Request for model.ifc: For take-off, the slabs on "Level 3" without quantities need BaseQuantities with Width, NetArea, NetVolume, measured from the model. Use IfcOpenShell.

First a look at what the model holds.

```python
import ifcopenshell
import ifcopenshell.util.element
import ifcopenshell.util.unit

model = ifcopenshell.open("model.ifc")
print(model.schema)
for unit_type in ("LENGTHUNIT", "AREAUNIT", "VOLUMEUNIT"):
    print(unit_type, ifcopenshell.util.unit.calculate_unit_scale(model, unit_type))
storey = next(s for s in model.by_type("IfcBuildingStorey") if s.Name == "Level 3")
slabs = [e for e in ifcopenshell.util.element.get_decomposition(storey) if e.is_a("IfcSlab")]
for e in sorted(slabs, key=lambda e: e.id()):
    print(e.id(), e.is_a(), e.Name, list(ifcopenshell.util.element.get_psets(e, qtos_only=True)), sep=" | ")
```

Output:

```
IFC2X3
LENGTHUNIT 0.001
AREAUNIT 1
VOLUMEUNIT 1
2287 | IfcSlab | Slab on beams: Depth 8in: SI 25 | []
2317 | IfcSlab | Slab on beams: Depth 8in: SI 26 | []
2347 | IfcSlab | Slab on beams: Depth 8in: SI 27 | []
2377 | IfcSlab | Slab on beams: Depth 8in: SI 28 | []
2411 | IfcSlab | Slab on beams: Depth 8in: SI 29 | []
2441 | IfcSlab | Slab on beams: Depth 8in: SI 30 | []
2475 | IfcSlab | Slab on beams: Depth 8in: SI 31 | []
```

```python
import ifcopenshell
import ifcopenshell.api.pset
import ifcopenshell.geom
import ifcopenshell.util.element
import ifcopenshell.util.shape
import ifcopenshell.util.unit

model = ifcopenshell.open("model.ifc")
unit_scale = ifcopenshell.util.unit.calculate_unit_scale(model)
area_scale = ifcopenshell.util.unit.calculate_unit_scale(model, "AREAUNIT")
volume_scale = ifcopenshell.util.unit.calculate_unit_scale(model, "VOLUMEUNIT")
settings = ifcopenshell.geom.settings()

storey = next(s for s in model.by_type("IfcBuildingStorey") if s.Name == "Level 3")
slabs = [e for e in ifcopenshell.util.element.get_decomposition(storey) if e.is_a("IfcSlab")]

for e in sorted(slabs, key=lambda e: e.id()):
    if ifcopenshell.util.element.get_psets(e, qtos_only=True, should_inherit=False):
        continue
    # Geometry comes back in metres, in the element's own axes.
    shape = ifcopenshell.geom.create_shape(settings, e)
    values = {
        "Width": ifcopenshell.util.shape.get_z(shape.geometry) / unit_scale,
        "NetArea": ifcopenshell.util.shape.get_footprint_area(shape.geometry) / area_scale,
        "NetVolume": ifcopenshell.util.shape.get_volume(shape.geometry) / volume_scale,
    }
    qto = ifcopenshell.api.pset.add_qto(model, product=e, name="BaseQuantities")
    ifcopenshell.api.pset.edit_qto(model, qto=qto, properties=values)
    print(e.id(), {k: round(v, 3) for k, v in values.items()})

model.write("model_v2.ifc")
```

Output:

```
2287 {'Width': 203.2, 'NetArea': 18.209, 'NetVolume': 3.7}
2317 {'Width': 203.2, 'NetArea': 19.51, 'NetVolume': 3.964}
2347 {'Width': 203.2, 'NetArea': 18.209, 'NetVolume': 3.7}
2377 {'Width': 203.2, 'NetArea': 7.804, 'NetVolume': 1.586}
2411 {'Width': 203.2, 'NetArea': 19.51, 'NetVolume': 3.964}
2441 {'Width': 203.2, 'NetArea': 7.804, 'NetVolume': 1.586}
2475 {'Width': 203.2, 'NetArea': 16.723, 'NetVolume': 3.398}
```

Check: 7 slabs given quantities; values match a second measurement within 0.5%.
